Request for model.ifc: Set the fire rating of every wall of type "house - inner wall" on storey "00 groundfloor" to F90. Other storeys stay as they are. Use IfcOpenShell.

First a look at what the model holds.

```python
import ifcopenshell
import ifcopenshell.util.element

model = ifcopenshell.open("model.ifc")
print(model.schema)
storey = next(s for s in model.by_type("IfcBuildingStorey") if s.Name == "00 groundfloor")
walls = [e for e in ifcopenshell.util.element.get_decomposition(storey) if e.is_a("IfcWall")]
seen = {}
for e in walls:
    element_type = ifcopenshell.util.element.get_type(e)
    key = (element_type.Name if element_type != e and element_type else None, ifcopenshell.util.element.get_pset(e, "Pset_WallCommon", "FireRating"))
    seen[key] = seen.get(key, 0) + 1
for (name, value), count in sorted(seen.items(), key=str):
    print(count, "x", name, "|", value)
```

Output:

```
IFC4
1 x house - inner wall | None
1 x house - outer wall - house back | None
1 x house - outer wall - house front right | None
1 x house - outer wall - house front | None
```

```python
import ifcopenshell
import ifcopenshell.api.pset
import ifcopenshell.util.element

model = ifcopenshell.open("model.ifc")

storey = next(s for s in model.by_type("IfcBuildingStorey") if s.Name == "00 groundfloor")
walls = [e for e in ifcopenshell.util.element.get_decomposition(storey) if e.is_a("IfcWall")]

count = 0
for e in walls:
    element_type = ifcopenshell.util.element.get_type(e)
    if element_type in (None, e) or element_type.Name != "house - inner wall":
        continue
    # add_pset returns the element's existing set when there is one.
    pset = ifcopenshell.api.pset.add_pset(model, product=e, name="Pset_WallCommon")
    ifcopenshell.api.pset.edit_pset(model, pset=pset, properties={"FireRating": "F90"})
    count += 1

print(count, "walls updated")

model.write("model_v2.ifc")
```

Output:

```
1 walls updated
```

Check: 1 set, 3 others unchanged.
